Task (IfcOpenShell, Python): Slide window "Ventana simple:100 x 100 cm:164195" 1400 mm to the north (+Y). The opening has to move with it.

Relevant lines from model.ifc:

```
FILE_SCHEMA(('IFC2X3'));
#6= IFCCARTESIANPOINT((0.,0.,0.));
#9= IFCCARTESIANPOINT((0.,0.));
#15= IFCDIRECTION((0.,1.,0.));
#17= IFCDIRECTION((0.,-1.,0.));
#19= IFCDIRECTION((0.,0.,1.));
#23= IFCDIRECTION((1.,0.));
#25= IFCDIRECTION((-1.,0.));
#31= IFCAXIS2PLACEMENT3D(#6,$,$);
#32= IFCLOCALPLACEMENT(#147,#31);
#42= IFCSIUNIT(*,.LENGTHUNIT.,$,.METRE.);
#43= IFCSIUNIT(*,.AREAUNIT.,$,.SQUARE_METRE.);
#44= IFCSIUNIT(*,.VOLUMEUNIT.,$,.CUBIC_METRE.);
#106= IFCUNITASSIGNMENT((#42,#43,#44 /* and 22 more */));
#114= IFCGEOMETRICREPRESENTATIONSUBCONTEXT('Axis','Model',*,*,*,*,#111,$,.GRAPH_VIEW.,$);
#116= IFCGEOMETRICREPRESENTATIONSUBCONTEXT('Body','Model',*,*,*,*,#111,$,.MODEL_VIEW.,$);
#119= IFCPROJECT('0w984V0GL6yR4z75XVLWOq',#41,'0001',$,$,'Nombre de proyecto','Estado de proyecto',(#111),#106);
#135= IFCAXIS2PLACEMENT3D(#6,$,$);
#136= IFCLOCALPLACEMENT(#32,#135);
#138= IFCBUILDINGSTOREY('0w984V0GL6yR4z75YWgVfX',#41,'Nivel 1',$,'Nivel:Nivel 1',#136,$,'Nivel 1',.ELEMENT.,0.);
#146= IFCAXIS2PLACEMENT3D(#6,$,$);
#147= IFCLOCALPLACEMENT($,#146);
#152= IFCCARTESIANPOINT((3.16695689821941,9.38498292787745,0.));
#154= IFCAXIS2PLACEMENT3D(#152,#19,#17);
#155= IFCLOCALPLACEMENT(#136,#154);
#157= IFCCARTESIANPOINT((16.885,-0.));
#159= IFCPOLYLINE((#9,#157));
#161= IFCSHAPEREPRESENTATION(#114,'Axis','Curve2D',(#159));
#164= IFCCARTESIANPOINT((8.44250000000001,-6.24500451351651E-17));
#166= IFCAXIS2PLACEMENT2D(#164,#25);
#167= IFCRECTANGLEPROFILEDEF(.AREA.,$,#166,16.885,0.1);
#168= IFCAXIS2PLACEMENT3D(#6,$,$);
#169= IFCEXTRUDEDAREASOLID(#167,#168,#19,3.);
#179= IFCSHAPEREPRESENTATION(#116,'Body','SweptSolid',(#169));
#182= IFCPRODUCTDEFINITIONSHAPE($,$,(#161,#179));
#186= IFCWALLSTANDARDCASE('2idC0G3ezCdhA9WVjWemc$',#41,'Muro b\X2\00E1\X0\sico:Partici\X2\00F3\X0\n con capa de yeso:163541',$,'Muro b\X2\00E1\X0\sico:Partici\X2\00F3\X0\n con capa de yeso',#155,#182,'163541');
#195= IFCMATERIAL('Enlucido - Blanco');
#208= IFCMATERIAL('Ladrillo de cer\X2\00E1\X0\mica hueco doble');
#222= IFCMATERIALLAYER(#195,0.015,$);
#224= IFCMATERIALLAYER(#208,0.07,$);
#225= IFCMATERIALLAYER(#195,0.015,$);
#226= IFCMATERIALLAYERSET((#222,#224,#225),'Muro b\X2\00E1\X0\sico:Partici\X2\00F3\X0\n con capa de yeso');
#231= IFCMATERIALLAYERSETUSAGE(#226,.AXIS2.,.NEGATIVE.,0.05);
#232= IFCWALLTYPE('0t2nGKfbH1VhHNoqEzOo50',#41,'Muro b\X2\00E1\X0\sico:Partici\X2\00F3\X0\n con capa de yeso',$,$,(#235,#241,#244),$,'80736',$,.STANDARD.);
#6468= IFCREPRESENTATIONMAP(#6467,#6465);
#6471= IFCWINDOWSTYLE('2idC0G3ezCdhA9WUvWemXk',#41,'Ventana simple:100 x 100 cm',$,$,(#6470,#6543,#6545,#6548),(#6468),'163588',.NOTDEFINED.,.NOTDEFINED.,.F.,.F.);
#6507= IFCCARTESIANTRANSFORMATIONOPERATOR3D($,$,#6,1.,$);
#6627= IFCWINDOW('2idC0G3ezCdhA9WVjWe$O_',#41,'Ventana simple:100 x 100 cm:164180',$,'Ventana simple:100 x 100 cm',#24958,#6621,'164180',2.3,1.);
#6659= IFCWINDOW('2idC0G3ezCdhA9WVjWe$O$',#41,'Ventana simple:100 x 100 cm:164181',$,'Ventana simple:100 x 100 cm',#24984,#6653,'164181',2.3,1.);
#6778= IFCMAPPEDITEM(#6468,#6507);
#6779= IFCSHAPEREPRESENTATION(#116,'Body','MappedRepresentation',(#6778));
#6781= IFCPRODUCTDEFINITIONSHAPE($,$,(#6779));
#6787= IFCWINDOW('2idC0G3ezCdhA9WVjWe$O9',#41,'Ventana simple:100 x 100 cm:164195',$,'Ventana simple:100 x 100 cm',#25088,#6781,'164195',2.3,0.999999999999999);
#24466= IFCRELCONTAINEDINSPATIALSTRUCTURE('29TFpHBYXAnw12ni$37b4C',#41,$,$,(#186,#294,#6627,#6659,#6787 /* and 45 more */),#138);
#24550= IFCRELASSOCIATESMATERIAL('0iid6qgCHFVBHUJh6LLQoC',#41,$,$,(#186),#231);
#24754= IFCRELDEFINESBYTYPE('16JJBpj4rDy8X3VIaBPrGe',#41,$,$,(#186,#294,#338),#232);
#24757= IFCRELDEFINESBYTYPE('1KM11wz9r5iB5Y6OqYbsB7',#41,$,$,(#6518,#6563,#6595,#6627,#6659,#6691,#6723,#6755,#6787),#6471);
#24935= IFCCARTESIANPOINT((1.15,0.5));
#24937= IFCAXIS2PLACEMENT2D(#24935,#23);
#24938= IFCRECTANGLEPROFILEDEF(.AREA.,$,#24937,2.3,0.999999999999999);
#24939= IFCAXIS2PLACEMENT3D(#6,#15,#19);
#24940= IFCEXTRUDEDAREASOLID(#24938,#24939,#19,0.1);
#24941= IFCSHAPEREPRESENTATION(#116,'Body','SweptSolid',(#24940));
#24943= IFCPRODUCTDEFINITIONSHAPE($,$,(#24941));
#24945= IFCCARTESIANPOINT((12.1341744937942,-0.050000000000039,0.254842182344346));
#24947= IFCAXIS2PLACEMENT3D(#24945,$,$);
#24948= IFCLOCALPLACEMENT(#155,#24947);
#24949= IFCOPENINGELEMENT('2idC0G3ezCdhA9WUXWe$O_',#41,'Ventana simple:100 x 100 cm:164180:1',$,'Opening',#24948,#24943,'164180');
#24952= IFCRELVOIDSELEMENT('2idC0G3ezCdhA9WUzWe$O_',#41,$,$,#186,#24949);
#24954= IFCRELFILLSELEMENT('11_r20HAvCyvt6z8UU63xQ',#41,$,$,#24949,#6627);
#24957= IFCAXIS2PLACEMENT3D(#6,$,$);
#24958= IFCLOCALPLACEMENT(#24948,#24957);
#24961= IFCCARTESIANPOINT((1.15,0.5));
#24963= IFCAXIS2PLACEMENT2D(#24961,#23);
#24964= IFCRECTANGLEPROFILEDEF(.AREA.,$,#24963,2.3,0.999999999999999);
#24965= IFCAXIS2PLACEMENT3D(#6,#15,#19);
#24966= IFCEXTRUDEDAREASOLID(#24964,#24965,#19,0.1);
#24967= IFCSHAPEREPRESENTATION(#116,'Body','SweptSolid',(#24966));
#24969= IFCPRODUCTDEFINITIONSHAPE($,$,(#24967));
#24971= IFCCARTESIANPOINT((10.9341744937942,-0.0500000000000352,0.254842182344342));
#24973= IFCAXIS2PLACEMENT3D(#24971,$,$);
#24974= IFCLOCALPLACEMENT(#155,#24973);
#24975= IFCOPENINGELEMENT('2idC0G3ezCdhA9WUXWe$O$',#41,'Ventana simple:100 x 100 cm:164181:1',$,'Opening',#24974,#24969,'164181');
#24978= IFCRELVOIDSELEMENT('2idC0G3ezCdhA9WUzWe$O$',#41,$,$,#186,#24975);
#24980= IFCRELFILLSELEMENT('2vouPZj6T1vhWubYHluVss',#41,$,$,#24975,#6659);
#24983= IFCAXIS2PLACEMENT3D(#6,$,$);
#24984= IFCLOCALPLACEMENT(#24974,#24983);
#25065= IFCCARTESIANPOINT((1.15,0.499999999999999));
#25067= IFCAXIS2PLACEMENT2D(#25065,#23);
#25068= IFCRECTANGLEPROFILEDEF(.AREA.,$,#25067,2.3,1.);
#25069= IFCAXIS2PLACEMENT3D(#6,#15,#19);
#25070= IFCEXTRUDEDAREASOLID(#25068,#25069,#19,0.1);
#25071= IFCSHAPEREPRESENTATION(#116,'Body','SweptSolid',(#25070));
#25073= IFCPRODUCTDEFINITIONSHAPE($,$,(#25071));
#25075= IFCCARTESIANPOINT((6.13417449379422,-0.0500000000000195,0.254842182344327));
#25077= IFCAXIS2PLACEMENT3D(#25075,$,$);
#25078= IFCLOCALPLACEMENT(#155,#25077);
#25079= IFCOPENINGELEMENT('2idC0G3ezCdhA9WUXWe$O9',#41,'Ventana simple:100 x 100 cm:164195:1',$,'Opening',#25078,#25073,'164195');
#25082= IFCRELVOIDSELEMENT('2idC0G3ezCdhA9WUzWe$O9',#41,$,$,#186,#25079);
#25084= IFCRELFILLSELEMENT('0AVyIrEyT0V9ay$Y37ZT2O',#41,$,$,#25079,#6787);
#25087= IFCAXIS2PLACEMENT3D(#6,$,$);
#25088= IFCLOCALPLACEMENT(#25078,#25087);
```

```python
import ifcopenshell
import ifcopenshell.api.geometry
import ifcopenshell.util.placement
import ifcopenshell.util.unit

model = ifcopenshell.open("model.ifc")
unit_scale = ifcopenshell.util.unit.calculate_unit_scale(model)

window = model.by_id(6787)
opening = window.FillsVoids[0].RelatingOpeningElement
wall = opening.VoidsElements[0].RelatingBuildingElement

wall_matrix = ifcopenshell.util.placement.get_local_placement(wall.ObjectPlacement)
shift = wall_matrix[:3, 0] * -1.4 / unit_scale
before = ifcopenshell.util.placement.get_local_placement(window.ObjectPlacement)[:3, 3].copy()

# The window is placed relative to its opening, so it follows when the opening moves.
matrix = ifcopenshell.util.placement.get_local_placement(opening.ObjectPlacement)
matrix[:3, 3] += shift
ifcopenshell.api.geometry.edit_object_placement(
    model, product=opening, matrix=matrix, is_si=False, should_transform_children=True
)

after = ifcopenshell.util.placement.get_local_placement(window.ObjectPlacement)[:3, 3]
print("window moved by", (after - before).round(3) + 0.0)

model.write("model_v2.ifc")
```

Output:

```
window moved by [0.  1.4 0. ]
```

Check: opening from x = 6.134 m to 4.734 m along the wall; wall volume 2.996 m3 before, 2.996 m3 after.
